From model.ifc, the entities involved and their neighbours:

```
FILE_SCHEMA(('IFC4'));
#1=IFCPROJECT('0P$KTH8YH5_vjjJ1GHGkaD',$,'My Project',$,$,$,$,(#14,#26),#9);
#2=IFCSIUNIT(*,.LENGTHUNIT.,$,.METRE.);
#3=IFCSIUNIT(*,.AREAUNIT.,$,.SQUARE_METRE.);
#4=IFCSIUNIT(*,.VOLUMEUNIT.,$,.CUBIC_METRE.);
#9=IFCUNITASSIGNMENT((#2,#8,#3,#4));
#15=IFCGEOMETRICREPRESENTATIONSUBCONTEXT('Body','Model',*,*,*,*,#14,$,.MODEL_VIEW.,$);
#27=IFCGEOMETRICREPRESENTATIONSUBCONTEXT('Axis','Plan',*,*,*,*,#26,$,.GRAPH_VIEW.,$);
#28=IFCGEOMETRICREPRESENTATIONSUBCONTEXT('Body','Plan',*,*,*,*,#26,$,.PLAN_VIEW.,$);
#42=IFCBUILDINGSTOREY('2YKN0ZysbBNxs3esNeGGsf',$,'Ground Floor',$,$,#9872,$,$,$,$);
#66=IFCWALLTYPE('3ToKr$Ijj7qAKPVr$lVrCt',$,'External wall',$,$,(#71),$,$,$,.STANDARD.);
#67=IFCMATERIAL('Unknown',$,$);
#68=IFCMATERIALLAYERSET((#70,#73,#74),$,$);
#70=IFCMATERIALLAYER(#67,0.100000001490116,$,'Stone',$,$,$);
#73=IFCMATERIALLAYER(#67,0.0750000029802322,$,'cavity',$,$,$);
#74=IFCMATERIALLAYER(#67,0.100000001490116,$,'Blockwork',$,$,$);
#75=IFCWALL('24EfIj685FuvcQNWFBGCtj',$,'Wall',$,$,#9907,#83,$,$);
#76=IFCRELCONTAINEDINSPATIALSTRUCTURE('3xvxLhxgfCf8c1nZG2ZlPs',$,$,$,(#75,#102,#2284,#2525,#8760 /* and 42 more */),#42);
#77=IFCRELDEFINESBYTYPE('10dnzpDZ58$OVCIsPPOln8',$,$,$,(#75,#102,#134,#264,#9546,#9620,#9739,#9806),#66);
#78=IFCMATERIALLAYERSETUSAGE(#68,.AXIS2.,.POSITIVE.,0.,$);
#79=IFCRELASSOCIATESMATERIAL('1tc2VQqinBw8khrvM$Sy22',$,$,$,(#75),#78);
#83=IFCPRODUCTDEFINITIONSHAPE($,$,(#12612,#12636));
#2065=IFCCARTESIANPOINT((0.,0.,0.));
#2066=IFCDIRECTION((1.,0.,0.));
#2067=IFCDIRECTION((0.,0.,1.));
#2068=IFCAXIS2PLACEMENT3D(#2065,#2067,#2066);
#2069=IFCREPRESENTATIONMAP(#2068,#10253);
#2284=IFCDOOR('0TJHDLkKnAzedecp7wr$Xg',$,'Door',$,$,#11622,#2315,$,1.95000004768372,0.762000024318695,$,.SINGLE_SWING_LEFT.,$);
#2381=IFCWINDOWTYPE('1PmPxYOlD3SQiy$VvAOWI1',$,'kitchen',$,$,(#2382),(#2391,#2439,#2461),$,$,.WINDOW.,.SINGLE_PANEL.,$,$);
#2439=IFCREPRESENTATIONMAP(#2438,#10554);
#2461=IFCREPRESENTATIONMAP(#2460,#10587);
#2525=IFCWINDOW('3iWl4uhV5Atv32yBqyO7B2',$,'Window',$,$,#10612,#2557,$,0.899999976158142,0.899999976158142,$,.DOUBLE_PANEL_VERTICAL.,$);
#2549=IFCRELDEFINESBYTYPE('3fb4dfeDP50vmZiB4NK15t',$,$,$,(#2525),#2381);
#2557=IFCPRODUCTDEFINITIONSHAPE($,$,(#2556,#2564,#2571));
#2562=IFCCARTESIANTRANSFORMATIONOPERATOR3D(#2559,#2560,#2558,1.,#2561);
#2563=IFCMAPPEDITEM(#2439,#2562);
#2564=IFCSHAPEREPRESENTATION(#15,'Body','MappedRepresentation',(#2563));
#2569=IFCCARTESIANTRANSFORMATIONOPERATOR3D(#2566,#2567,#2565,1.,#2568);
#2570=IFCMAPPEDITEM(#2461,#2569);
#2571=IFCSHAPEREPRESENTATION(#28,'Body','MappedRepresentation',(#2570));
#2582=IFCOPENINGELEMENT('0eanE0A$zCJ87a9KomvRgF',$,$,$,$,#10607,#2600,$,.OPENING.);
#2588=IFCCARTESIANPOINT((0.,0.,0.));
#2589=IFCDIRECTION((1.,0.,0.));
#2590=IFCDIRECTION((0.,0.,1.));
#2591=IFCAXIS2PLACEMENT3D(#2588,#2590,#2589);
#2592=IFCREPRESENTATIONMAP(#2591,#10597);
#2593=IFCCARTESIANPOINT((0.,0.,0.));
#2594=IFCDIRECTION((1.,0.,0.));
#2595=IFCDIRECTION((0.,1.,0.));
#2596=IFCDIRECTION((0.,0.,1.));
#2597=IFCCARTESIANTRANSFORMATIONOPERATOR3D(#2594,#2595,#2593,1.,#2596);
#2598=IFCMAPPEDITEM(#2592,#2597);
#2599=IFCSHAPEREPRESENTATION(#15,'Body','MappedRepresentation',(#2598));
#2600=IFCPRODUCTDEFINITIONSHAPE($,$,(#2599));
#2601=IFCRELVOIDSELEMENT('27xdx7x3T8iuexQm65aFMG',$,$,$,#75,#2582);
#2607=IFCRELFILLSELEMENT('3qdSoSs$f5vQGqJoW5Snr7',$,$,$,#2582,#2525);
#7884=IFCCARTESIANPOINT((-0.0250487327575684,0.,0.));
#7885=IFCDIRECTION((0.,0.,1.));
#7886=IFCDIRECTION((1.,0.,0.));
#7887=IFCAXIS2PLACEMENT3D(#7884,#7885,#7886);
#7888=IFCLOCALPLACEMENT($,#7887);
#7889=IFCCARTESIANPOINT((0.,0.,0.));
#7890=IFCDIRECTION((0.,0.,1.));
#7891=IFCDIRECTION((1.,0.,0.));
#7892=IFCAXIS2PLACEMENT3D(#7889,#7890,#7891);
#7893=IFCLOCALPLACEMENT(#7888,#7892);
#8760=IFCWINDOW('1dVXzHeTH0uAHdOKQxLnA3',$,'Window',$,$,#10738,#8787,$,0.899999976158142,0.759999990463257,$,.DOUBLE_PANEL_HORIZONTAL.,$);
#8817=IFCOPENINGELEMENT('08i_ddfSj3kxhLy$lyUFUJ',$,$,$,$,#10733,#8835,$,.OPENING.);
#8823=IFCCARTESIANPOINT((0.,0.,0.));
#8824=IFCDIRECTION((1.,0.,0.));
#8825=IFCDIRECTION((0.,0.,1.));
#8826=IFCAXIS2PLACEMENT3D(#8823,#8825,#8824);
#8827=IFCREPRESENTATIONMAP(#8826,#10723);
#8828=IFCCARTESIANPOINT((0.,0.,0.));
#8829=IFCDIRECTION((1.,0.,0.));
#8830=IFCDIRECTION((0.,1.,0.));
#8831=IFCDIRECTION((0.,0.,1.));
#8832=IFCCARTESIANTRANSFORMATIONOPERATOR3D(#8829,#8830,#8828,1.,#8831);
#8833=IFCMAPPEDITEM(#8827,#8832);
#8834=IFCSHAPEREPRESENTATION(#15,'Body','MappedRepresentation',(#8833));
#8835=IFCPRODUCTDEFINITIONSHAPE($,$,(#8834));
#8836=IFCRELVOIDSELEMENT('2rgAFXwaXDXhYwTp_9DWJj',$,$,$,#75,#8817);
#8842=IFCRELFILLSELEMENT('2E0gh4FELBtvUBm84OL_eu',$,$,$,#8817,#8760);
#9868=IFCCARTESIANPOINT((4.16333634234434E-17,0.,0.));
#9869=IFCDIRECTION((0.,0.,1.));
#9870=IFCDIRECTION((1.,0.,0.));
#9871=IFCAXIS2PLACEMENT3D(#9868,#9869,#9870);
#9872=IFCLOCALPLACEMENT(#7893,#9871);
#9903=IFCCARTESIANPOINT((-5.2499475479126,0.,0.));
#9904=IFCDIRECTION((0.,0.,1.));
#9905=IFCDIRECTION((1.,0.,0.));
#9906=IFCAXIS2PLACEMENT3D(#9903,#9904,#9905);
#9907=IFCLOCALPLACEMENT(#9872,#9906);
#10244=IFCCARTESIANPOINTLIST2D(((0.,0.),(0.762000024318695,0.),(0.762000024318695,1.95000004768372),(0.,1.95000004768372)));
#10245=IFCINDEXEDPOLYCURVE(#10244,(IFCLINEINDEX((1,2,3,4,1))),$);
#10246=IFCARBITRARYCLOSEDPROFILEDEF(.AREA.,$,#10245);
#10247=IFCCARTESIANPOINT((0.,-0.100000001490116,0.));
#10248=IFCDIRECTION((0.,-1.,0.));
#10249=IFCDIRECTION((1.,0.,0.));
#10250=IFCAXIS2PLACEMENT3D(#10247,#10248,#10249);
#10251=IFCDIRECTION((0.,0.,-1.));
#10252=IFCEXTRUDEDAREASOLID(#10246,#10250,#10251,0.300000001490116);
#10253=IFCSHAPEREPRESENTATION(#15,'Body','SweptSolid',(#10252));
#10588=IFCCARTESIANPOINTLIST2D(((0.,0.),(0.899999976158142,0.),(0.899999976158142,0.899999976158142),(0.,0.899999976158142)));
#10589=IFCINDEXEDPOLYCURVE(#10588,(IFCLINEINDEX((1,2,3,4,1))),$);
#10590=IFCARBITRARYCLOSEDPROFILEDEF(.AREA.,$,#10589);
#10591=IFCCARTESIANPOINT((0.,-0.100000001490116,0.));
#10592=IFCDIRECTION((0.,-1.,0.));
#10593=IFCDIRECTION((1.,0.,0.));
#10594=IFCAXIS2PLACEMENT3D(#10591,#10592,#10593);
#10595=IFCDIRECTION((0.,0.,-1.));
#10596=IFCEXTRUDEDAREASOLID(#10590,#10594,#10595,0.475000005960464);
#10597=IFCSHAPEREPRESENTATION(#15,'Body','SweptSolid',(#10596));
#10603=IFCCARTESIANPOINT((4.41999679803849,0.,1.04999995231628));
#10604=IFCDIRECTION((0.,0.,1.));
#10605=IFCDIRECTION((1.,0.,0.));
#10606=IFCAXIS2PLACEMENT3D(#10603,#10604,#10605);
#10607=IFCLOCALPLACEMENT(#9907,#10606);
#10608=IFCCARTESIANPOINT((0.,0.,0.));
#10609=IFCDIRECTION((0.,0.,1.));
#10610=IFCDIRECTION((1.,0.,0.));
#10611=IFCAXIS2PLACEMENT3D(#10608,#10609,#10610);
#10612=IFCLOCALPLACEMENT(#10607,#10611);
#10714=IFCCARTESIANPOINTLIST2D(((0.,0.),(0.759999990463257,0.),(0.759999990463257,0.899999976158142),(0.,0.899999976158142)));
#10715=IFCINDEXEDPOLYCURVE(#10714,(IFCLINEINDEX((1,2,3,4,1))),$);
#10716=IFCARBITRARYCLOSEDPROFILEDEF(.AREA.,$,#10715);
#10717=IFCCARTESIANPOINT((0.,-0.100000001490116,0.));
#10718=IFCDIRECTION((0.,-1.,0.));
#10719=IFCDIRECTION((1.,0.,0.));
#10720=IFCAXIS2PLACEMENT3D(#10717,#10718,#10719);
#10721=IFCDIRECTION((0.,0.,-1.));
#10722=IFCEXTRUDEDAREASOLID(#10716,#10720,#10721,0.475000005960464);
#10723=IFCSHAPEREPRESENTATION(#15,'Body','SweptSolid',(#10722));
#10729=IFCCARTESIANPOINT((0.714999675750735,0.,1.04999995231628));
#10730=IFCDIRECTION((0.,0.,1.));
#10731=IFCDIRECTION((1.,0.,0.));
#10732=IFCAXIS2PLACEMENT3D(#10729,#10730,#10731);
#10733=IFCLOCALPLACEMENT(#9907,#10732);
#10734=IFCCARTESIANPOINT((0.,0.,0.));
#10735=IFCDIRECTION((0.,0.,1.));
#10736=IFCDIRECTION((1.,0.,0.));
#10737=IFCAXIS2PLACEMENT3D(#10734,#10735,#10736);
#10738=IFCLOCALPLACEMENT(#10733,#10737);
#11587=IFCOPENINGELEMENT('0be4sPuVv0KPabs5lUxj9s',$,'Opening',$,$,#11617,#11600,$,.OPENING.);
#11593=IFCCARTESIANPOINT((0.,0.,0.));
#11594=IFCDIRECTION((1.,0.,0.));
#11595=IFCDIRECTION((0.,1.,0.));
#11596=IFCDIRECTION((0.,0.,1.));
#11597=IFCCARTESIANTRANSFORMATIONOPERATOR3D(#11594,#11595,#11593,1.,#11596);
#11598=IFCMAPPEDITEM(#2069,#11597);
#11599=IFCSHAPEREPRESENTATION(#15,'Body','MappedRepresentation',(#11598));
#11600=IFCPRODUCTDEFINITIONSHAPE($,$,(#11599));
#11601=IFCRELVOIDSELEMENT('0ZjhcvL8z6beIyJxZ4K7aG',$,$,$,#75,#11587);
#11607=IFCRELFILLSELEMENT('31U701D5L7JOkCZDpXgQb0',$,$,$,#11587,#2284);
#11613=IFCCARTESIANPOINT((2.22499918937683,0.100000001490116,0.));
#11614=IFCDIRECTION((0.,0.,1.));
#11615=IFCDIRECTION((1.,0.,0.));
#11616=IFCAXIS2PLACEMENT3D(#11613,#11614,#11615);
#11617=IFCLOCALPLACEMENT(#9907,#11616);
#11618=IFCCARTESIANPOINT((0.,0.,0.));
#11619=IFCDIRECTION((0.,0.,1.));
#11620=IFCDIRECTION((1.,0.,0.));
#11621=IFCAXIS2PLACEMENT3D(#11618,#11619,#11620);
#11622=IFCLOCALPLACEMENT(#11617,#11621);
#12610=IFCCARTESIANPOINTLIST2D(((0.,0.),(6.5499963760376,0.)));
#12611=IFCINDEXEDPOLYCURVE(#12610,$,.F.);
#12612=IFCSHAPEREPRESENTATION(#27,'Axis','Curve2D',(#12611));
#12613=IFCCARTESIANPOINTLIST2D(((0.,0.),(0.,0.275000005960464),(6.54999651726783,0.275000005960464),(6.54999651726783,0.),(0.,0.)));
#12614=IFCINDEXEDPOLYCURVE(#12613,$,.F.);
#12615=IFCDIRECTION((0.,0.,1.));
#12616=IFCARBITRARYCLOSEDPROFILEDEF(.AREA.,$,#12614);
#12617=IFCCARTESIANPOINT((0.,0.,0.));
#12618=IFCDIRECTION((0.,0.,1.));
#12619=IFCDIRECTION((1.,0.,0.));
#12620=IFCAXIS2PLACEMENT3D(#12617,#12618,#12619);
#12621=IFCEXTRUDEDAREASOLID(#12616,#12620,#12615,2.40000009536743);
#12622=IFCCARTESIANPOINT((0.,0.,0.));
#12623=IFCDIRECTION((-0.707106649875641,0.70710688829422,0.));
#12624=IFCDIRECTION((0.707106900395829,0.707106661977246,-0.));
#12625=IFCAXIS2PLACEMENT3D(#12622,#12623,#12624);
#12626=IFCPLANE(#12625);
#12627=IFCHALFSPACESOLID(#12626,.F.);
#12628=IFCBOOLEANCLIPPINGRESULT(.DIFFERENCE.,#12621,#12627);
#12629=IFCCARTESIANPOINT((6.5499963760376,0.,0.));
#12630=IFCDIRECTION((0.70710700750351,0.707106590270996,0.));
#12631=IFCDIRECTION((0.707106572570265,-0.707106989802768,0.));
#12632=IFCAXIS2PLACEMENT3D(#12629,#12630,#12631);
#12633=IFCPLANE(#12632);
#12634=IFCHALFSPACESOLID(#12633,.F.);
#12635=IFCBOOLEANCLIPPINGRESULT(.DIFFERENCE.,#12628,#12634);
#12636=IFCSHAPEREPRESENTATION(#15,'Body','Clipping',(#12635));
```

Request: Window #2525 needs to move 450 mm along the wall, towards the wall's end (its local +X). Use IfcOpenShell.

```python
import ifcopenshell
import ifcopenshell.api.geometry
import ifcopenshell.util.placement

model = ifcopenshell.open("model.ifc")

window = model.by_guid("3iWl4uhV5Atv32yBqyO7B2")
opening = window.FillsVoids[0].RelatingOpeningElement
wall = opening.VoidsElements[0].RelatingBuildingElement

wall_matrix = ifcopenshell.util.placement.get_local_placement(wall.ObjectPlacement)
shift = wall_matrix[:3, 0] * 0.45
before = ifcopenshell.util.placement.get_local_placement(window.ObjectPlacement)[:3, 3].copy()

# The window is placed relative to its opening, so it follows when the opening moves.
matrix = ifcopenshell.util.placement.get_local_placement(opening.ObjectPlacement)
matrix[:3, 3] += shift
ifcopenshell.api.geometry.edit_object_placement(
    model, product=opening, matrix=matrix, is_si=False, should_transform_children=True
)

after = ifcopenshell.util.placement.get_local_placement(window.ObjectPlacement)[:3, 3]
print("window moved by", (after - before).round(3) + 0.0)

model.write("model_updated.ifc")
```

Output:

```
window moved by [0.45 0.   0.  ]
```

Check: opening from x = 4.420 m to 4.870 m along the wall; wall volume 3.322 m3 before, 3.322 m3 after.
